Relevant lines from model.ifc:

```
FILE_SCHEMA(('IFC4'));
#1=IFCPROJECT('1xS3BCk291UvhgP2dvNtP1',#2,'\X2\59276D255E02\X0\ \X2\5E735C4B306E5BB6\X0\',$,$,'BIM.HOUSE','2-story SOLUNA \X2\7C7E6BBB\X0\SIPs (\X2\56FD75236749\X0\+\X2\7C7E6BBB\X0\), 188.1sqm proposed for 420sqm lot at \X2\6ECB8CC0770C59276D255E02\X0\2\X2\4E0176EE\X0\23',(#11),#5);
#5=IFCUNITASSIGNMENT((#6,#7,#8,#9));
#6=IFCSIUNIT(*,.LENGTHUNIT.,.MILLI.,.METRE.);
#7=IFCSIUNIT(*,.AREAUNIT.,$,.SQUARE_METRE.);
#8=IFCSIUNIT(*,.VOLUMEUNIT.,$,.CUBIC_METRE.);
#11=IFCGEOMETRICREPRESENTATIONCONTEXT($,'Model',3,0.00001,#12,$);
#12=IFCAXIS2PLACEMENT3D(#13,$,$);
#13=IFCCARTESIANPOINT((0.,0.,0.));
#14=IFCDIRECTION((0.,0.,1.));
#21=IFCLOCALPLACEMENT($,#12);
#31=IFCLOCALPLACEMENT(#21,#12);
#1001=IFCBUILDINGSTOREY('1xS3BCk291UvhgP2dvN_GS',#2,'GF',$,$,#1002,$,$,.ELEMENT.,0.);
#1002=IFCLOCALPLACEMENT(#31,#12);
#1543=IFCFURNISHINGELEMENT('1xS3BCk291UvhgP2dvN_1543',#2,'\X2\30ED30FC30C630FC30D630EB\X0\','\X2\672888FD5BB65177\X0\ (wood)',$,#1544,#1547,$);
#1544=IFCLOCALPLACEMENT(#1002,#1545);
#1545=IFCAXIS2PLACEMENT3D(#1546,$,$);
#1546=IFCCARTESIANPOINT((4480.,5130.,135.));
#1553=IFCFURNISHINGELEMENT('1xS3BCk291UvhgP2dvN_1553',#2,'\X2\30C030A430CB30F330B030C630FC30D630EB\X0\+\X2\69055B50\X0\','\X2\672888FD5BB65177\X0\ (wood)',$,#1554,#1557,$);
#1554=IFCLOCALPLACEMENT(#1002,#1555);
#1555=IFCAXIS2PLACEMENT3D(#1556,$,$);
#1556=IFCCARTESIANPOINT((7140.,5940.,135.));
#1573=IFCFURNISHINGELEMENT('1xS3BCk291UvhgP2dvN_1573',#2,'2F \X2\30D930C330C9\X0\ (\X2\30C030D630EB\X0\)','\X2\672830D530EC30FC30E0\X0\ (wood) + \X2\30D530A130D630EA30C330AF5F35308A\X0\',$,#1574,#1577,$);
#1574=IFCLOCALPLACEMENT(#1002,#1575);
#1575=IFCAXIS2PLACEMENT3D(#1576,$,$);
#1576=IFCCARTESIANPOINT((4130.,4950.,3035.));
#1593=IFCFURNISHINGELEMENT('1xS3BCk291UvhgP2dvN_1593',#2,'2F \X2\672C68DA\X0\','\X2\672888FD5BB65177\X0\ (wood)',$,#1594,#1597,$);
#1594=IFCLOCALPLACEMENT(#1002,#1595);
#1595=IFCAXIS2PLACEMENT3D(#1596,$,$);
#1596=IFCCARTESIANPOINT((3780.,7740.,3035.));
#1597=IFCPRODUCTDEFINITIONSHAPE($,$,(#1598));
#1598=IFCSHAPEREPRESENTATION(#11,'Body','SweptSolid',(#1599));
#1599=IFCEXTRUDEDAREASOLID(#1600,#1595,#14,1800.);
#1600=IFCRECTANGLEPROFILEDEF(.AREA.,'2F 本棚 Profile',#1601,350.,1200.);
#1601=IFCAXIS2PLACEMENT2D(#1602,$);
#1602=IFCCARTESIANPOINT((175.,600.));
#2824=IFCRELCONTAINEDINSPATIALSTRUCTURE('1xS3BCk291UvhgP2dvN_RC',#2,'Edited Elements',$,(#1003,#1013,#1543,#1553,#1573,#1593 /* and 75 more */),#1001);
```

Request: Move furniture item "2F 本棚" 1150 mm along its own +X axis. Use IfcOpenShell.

```python
import ifcopenshell
import ifcopenshell.api.geometry
import ifcopenshell.util.placement
import ifcopenshell.util.unit

model = ifcopenshell.open("model.ifc")
unit_scale = ifcopenshell.util.unit.calculate_unit_scale(model)

item = model.by_guid("1xS3BCk291UvhgP2dvN_1593")
matrix = ifcopenshell.util.placement.get_local_placement(item.ObjectPlacement)
matrix[:3, 3] += matrix[:3, 0] * 1.15 / unit_scale
ifcopenshell.api.geometry.edit_object_placement(model, product=item, matrix=matrix, is_si=False)

print(ifcopenshell.util.placement.get_local_placement(item.ObjectPlacement).round(3) + 0.0)

model.write("model_v2.ifc")
```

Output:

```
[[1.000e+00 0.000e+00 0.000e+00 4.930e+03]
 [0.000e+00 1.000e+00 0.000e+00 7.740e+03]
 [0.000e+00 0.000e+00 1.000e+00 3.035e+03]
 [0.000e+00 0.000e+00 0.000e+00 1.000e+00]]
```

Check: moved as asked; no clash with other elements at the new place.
